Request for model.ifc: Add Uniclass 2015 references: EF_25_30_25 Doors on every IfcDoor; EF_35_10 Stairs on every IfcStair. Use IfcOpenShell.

First a look at what the model holds.

```python
import ifcopenshell

model = ifcopenshell.open("model.ifc")
print(model.schema)
print("classifications:", [c.Name for c in model.by_type("IfcClassification")])
for ifc_class in ("IfcDoor", "IfcRoof", "IfcStair", "IfcWall", "IfcWindow"):
    print(ifc_class, len(model.by_type(ifc_class)))
```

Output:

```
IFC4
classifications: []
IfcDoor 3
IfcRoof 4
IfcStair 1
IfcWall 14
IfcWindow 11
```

```python
import ifcopenshell
import ifcopenshell.api.classification

model = ifcopenshell.open("model.ifc")

system = ifcopenshell.api.classification.add_classification(model, classification="Uniclass 2015")

codes = {
    "IfcDoor": ("EF_25_30_25", "Doors"),
    "IfcStair": ("EF_35_10", "Stairs"),
}
for ifc_class, (code, name) in codes.items():
    products = model.by_type(ifc_class)
    ifcopenshell.api.classification.add_reference(
        model, products=products, classification=system, identification=code, name=name
    )
    print(code, len(products))

model.write("model-out.ifc")
```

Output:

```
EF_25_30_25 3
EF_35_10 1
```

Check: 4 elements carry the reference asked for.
